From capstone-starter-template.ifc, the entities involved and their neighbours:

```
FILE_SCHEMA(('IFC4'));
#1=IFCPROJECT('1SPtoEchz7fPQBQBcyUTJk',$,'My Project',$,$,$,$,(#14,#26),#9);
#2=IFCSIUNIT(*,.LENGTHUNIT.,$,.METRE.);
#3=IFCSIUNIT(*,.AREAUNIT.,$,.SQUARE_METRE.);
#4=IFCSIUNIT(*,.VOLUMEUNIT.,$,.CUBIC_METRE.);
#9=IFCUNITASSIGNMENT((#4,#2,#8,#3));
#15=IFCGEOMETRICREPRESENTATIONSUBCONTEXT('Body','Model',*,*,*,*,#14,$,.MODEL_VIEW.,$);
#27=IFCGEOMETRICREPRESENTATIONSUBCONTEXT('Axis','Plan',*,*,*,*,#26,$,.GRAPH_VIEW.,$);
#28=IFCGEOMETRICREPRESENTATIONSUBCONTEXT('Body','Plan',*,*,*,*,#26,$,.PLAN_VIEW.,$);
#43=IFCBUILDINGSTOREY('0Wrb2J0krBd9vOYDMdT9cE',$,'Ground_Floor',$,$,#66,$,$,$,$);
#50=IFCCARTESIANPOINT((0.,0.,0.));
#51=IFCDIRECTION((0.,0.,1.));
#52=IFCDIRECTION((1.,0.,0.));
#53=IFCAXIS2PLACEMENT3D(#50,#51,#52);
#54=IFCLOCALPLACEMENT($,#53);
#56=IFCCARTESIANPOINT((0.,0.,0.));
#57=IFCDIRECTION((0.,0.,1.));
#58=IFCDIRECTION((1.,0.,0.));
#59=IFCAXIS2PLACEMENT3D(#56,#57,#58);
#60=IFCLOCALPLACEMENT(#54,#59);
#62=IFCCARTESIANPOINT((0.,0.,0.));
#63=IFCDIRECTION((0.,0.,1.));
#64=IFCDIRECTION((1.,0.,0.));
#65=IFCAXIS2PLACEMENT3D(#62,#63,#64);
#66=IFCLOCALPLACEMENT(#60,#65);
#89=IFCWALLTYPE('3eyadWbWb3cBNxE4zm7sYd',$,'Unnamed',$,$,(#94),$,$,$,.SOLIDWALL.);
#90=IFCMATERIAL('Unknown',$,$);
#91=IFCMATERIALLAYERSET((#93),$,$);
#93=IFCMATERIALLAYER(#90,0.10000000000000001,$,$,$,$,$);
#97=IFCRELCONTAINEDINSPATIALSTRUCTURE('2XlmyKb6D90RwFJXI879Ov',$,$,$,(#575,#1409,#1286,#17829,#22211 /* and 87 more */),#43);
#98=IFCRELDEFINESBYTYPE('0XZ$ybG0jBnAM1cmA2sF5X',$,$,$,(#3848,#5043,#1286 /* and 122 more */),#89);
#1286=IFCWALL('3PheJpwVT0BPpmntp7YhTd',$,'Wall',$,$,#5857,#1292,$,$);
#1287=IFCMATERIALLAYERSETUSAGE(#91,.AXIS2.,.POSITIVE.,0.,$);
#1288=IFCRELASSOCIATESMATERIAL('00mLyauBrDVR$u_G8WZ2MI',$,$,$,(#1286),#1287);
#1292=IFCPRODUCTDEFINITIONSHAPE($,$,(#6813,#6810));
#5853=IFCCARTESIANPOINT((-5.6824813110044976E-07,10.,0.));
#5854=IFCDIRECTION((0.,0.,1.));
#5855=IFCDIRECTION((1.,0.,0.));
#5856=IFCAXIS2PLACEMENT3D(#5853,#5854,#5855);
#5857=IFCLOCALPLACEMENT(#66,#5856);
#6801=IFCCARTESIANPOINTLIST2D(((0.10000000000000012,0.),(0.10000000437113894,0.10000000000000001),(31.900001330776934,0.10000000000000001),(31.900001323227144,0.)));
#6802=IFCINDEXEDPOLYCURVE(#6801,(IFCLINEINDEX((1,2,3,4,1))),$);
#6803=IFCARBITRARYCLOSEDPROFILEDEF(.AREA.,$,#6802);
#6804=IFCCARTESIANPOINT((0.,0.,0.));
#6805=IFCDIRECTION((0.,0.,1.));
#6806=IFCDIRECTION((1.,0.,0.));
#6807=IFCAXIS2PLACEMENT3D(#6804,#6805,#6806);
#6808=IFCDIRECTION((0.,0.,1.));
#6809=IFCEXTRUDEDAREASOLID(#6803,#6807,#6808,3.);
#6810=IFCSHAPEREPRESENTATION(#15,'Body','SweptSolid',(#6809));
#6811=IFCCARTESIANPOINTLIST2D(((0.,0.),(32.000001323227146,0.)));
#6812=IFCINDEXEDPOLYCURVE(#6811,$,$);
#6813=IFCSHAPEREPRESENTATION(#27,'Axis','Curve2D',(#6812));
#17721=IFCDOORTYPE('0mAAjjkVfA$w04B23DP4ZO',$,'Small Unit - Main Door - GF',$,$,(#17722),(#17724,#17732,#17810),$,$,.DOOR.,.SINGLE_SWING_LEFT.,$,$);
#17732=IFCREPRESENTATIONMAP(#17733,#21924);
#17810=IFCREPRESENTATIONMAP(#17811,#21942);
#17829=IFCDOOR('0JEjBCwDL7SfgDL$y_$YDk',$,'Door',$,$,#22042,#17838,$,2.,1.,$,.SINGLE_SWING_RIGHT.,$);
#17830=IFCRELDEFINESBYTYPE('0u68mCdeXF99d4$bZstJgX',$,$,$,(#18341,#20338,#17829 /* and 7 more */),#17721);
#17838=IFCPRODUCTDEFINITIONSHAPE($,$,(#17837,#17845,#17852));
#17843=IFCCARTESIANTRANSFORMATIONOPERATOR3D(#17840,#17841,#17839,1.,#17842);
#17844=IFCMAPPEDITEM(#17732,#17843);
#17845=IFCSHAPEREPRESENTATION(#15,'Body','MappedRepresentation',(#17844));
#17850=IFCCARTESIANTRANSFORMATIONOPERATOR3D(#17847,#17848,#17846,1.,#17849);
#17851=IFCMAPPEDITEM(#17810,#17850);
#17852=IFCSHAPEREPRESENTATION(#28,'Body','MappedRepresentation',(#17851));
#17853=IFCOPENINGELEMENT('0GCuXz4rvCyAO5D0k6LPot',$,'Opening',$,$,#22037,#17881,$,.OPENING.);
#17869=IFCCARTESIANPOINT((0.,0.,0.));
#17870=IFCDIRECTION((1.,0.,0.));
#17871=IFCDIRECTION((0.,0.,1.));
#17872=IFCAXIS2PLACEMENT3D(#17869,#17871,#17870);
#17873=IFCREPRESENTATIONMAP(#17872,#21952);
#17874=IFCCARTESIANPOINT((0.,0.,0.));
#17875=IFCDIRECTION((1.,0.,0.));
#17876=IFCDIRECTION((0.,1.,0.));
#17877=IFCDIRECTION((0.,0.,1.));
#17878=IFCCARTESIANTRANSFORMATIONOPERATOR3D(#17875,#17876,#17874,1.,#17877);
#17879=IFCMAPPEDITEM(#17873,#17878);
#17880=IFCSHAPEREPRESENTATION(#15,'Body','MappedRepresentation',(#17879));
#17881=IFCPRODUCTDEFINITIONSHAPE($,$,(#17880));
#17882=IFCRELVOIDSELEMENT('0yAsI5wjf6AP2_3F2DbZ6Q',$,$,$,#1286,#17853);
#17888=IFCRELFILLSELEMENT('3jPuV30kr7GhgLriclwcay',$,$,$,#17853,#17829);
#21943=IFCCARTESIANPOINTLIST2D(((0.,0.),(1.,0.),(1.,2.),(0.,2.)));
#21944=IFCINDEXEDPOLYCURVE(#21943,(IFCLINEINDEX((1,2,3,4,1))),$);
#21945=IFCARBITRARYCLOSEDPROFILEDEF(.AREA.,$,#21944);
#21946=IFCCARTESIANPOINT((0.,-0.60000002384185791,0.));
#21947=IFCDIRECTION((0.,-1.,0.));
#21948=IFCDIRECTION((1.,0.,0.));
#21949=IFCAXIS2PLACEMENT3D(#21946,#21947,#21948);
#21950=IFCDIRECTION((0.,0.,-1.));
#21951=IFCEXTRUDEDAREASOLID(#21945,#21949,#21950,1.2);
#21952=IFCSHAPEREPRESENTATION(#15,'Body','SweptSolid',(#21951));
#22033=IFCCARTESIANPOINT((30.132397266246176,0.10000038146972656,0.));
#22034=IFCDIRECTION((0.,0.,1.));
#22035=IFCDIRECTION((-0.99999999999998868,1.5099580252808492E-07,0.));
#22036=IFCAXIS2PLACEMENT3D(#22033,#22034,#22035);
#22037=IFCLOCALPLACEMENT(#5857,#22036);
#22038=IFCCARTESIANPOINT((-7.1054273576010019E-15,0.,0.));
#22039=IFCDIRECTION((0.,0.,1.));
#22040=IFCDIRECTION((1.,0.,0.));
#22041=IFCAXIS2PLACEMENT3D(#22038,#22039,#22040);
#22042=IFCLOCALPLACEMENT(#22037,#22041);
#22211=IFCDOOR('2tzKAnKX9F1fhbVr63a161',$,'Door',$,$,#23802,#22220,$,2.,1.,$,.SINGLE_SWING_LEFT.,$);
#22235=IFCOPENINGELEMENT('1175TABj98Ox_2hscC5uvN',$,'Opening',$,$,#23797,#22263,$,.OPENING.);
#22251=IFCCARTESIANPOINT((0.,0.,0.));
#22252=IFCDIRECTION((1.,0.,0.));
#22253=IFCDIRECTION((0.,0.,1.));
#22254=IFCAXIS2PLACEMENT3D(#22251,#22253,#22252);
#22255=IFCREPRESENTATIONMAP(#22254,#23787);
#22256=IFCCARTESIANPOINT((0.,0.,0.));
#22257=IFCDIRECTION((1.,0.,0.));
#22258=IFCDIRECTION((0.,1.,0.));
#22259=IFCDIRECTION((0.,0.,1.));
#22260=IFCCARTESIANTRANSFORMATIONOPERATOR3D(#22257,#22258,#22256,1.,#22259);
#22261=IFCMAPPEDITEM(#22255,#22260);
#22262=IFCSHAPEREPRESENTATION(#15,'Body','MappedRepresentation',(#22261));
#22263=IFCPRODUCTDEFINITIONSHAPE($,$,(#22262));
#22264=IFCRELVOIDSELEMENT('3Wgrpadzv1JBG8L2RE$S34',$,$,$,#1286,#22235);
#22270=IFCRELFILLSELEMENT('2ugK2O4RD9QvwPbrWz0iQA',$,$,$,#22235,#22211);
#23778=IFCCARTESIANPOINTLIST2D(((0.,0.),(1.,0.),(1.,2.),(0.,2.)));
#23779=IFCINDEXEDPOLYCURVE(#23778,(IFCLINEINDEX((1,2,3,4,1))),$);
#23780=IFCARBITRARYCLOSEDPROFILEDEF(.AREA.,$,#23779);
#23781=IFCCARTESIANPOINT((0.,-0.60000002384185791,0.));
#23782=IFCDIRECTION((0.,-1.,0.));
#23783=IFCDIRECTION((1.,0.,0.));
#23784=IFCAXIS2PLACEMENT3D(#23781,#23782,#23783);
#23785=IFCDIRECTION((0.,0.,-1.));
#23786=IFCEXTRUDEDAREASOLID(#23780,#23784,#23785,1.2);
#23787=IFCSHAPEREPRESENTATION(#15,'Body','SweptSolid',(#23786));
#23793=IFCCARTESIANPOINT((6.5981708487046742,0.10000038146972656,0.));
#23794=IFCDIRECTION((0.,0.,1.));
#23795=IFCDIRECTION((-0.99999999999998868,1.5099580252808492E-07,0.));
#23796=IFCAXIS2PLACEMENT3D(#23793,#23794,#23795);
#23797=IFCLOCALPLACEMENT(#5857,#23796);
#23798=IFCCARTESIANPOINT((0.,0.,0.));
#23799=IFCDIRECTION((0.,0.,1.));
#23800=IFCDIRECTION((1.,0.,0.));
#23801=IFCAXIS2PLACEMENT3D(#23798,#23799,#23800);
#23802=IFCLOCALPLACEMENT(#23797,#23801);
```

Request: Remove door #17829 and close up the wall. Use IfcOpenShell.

```python
import ifcopenshell
import ifcopenshell.api.feature
import ifcopenshell.api.root
import ifcopenshell.geom
import ifcopenshell.util.shape

model = ifcopenshell.open("capstone-starter-template.ifc")
settings = ifcopenshell.geom.settings()


def volume(element):
    """Net volume in cubic metres, openings subtracted."""
    shape = ifcopenshell.geom.create_shape(settings, element)
    return ifcopenshell.util.shape.get_volume(shape.geometry)


door = model.by_id(17829)
opening = door.FillsVoids[0].RelatingOpeningElement
wall = opening.VoidsElements[0].RelatingBuildingElement
before = volume(wall)

ifcopenshell.api.root.remove_product(model, product=door)
ifcopenshell.api.feature.remove_feature(model, feature=opening)

after = volume(wall)

print(f"wall volume {before:.3f} -> {after:.3f} m3")

model.write("capstone-starter-template_v2.ifc")
```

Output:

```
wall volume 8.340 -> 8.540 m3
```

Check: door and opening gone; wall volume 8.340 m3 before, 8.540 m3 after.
